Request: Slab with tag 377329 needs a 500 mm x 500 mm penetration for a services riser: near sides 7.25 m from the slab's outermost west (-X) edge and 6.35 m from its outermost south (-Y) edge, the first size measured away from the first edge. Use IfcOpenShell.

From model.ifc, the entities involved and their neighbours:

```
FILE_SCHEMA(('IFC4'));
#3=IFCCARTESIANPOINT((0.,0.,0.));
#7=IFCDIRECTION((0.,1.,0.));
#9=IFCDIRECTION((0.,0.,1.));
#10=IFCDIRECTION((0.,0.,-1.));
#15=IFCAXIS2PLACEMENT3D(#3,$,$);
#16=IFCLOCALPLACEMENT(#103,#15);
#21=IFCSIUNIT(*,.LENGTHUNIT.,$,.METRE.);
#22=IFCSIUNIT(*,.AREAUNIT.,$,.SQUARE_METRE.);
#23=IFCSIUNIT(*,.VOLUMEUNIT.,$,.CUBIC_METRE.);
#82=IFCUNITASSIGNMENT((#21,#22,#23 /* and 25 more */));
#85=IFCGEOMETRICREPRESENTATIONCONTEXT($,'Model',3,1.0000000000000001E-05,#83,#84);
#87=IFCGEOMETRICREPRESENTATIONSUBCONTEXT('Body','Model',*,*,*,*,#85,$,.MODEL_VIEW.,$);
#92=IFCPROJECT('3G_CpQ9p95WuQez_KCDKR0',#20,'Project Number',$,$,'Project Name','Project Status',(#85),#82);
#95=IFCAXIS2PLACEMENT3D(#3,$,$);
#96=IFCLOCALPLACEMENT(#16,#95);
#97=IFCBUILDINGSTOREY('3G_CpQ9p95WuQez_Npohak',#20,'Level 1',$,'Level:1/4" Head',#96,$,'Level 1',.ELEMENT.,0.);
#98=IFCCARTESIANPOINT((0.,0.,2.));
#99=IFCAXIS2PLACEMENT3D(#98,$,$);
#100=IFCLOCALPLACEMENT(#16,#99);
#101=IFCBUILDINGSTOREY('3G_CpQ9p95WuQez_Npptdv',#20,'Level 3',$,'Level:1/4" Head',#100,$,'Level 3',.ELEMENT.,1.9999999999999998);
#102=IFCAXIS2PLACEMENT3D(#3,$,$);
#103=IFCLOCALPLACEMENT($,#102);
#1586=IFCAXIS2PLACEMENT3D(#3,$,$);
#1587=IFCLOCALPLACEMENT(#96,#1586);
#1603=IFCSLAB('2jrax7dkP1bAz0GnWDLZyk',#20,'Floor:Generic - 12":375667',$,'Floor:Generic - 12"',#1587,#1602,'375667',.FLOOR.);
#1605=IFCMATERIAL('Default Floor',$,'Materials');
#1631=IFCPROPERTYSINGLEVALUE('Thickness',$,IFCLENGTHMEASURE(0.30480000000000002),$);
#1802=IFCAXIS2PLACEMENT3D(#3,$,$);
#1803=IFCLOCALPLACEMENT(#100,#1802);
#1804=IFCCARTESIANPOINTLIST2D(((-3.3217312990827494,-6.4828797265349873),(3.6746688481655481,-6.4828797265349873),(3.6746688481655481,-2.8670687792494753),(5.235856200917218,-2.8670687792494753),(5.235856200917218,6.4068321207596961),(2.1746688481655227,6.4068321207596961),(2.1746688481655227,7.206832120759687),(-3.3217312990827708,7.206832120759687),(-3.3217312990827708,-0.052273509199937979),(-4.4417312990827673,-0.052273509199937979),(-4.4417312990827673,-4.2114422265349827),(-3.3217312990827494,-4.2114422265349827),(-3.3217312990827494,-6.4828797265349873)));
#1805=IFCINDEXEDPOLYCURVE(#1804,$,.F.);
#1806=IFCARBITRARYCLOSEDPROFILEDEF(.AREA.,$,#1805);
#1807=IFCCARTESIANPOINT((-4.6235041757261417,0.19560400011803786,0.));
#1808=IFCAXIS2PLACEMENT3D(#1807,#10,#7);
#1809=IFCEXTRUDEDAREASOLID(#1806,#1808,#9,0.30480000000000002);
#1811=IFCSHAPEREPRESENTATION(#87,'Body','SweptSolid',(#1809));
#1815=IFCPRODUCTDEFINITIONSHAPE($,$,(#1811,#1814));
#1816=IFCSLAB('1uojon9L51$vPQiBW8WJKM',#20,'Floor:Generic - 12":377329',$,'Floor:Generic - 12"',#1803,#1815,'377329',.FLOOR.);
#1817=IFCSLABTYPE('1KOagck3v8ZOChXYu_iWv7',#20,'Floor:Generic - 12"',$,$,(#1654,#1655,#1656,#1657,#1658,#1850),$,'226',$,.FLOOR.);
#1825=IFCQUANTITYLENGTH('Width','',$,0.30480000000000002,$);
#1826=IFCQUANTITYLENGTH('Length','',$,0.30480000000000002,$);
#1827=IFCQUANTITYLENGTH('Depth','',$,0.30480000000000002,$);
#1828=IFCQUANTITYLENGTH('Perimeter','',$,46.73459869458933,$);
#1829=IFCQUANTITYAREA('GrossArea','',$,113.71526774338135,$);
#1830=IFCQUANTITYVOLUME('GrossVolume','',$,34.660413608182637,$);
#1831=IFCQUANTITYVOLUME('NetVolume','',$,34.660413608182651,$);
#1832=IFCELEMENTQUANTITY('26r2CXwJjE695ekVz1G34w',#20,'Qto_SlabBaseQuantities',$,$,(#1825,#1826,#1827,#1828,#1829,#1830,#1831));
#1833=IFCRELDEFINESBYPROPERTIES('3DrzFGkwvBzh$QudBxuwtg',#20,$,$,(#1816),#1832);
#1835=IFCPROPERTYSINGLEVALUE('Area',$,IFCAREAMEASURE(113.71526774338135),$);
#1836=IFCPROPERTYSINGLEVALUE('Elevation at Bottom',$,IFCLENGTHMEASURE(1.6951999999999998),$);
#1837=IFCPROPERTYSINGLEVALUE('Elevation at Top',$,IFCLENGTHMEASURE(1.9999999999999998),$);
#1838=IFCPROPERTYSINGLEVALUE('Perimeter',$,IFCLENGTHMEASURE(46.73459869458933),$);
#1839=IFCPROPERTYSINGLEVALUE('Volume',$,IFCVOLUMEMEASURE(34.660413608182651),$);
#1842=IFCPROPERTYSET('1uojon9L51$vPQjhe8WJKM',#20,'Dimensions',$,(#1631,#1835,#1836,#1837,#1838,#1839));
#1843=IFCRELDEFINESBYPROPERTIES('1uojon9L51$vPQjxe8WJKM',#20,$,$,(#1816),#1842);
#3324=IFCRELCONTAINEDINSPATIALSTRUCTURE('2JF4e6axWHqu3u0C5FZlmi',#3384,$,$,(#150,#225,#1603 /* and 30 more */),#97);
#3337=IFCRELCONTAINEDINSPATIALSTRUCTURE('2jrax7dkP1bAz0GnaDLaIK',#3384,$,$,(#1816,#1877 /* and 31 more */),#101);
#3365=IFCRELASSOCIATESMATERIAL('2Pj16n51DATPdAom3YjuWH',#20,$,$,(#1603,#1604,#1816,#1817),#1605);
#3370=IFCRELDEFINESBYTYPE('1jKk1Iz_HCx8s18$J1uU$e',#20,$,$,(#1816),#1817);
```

```python
import numpy as np
import ifcopenshell
import ifcopenshell.api.feature
import ifcopenshell.api.geometry
import ifcopenshell.api.pset
import ifcopenshell.api.root
import ifcopenshell.geom
import ifcopenshell.util.element
import ifcopenshell.util.placement
import ifcopenshell.util.representation
import ifcopenshell.util.shape
import ifcopenshell.util.unit

model = ifcopenshell.open("model.ifc")
unit_scale = ifcopenshell.util.unit.calculate_unit_scale(model)
area_scale = ifcopenshell.util.unit.calculate_unit_scale(model, "AREAUNIT")
volume_scale = ifcopenshell.util.unit.calculate_unit_scale(model, "VOLUMEUNIT")
settings = ifcopenshell.geom.settings()


def volume(element):
    """Net volume in cubic metres, openings subtracted."""
    shape = ifcopenshell.geom.create_shape(settings, element)
    return ifcopenshell.util.shape.get_volume(shape.geometry)


slab = model.by_guid("1uojon9L51$vPQiBW8WJKM")
before = volume(slab)

# Extent in the slab's own axes, in metres. The edges named are its -X and -Y sides.
slab_shape = ifcopenshell.geom.create_shape(settings, slab)
vertices = ifcopenshell.util.shape.get_vertices(slab_shape.geometry)
x_min, y_min, bottom = vertices.min(axis=0)
top = vertices[:, 2].max()

opening = ifcopenshell.api.root.create_entity(model, ifc_class="IfcOpeningElement", name="Services riser opening", predefined_type="OPENING")
context = ifcopenshell.util.representation.get_context(model, "Model", "Body", "MODEL_VIEW")
width, depth = 0.5, 0.5
outline = [(0.0, 0.0), (width, 0.0), (width, depth), (0.0, depth), (0.0, 0.0)]
# Overshoot both faces by 50 mm so the cut is clean.
shape = ifcopenshell.api.geometry.add_slab_representation(
    model, context=context, depth=top - bottom + 0.1, polyline=outline
)
ifcopenshell.api.geometry.assign_representation(model, product=opening, representation=shape)

matrix = ifcopenshell.util.placement.get_local_placement(slab.ObjectPlacement)
matrix[:, 3] = matrix @ np.append(np.array([x_min + 7.25, y_min + 6.35, bottom - 0.05]) / unit_scale, 1.0)
ifcopenshell.api.geometry.edit_object_placement(model, product=opening, matrix=matrix, is_si=False)
ifcopenshell.api.feature.add_feature(model, feature=opening, element=slab)

after = volume(slab)

# Update the slab's stored quantities.
qto = model.by_id(ifcopenshell.util.element.get_pset(slab, "Qto_SlabBaseQuantities", should_inherit=False)["id"])
ifcopenshell.api.pset.edit_qto(model, qto=qto, properties={"NetVolume": after / volume_scale})
pset = model.by_id(ifcopenshell.util.element.get_pset(slab, "Dimensions", should_inherit=False)["id"])
ifcopenshell.api.pset.edit_pset(model, pset=pset, properties={
    "Area": model.create_entity("IfcAreaMeasure", after / (top - bottom) / area_scale),
    "Volume": model.create_entity("IfcVolumeMeasure", after / volume_scale),
})

print(f"slab volume {before:.3f} -> {after:.3f} m3")

model.write("model_v2.ifc")
```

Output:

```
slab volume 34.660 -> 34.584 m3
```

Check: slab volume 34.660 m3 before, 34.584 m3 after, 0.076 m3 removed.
